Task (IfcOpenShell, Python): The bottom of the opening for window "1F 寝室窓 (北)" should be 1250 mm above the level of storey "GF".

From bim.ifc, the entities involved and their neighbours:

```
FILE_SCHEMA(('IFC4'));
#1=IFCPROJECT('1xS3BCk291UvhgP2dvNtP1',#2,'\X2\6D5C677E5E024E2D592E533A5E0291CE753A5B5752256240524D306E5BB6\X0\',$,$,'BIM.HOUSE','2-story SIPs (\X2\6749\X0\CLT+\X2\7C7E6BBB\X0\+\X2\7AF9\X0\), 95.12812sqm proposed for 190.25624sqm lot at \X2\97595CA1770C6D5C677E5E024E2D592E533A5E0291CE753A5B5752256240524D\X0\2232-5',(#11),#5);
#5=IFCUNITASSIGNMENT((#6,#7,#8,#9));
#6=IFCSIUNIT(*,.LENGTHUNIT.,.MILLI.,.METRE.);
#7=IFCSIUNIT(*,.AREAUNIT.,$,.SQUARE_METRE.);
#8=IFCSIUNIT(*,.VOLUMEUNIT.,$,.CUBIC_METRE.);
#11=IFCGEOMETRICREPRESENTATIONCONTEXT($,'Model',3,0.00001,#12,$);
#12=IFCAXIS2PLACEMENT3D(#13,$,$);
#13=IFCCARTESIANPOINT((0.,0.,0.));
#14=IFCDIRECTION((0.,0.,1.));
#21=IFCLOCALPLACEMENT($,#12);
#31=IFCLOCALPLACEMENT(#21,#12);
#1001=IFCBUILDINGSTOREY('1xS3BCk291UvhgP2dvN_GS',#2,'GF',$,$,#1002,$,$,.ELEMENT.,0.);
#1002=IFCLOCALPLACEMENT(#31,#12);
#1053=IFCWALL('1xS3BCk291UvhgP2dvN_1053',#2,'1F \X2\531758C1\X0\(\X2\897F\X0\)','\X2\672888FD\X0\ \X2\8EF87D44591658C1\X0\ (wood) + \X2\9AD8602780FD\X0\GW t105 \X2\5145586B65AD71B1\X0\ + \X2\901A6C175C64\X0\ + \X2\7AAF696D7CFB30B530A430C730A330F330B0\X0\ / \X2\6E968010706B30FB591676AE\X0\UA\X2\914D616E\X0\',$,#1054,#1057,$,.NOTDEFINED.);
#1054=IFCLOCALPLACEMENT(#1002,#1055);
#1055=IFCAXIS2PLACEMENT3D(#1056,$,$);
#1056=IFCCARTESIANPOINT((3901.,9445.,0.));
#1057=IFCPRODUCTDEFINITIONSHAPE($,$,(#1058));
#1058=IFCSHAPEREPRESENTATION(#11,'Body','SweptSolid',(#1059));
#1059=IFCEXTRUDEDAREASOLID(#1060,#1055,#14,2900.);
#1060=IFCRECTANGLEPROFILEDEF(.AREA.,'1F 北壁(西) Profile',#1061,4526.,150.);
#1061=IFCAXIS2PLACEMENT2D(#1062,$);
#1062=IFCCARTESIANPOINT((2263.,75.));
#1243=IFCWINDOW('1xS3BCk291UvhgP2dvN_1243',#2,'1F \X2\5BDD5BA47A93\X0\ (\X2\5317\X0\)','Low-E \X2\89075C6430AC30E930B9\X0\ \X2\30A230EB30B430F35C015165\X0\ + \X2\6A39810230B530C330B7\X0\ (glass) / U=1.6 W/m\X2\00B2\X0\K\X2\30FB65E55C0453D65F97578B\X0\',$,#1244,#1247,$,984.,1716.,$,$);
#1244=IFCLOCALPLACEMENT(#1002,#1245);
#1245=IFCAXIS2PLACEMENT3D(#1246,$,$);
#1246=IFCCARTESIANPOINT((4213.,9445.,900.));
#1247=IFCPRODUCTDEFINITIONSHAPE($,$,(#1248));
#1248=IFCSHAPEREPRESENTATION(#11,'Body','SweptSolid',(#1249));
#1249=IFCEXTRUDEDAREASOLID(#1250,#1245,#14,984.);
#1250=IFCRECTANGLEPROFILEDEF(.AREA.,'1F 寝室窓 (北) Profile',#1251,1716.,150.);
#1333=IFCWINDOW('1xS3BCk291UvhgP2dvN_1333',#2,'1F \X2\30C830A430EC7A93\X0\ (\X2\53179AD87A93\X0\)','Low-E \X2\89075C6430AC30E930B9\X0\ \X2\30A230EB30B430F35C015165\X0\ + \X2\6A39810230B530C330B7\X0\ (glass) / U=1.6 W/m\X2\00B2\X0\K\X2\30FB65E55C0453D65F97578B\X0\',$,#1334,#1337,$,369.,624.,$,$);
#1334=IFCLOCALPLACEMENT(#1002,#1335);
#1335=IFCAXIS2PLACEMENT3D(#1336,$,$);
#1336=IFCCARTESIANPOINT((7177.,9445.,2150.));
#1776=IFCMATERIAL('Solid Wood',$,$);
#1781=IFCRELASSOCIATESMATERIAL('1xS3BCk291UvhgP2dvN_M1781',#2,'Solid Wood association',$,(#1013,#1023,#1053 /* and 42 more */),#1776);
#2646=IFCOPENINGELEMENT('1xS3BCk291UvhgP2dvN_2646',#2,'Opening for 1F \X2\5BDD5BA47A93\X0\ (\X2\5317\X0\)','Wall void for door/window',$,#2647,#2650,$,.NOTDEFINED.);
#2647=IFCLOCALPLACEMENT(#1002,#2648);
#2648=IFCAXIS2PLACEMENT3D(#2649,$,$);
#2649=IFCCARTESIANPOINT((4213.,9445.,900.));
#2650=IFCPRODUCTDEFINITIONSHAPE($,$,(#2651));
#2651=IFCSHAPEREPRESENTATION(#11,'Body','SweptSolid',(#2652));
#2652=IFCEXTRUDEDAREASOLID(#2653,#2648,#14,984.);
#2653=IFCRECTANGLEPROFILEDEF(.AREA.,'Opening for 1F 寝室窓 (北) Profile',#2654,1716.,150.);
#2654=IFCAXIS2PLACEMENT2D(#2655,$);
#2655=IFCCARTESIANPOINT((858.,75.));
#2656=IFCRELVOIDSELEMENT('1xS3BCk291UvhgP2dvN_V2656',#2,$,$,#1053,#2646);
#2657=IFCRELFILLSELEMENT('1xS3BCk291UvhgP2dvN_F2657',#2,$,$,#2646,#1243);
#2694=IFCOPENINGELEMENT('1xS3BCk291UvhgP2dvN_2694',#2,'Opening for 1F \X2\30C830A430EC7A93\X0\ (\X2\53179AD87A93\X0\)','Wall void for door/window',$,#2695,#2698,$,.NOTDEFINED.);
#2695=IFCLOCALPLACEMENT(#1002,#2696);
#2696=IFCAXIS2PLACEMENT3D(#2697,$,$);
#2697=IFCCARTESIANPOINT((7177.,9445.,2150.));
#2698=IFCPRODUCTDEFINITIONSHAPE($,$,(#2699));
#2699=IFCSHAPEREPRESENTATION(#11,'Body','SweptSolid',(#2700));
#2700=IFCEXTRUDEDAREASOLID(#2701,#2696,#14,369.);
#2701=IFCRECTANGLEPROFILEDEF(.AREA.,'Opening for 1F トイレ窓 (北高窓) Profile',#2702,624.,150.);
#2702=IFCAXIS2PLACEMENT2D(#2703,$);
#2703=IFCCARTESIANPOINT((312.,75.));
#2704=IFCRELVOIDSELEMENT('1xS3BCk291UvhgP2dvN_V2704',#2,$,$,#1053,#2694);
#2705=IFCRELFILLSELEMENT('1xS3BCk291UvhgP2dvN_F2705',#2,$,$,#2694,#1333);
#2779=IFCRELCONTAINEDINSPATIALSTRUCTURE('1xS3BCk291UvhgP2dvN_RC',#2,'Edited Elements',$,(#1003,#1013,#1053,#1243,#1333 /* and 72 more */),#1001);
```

```python
import numpy as np
import ifcopenshell
import ifcopenshell.api.geometry
import ifcopenshell.geom
import ifcopenshell.util.element
import ifcopenshell.util.placement
import ifcopenshell.util.shape
import ifcopenshell.util.unit

model = ifcopenshell.open("bim.ifc")
unit_scale = ifcopenshell.util.unit.calculate_unit_scale(model)

window = model.by_guid("1xS3BCk291UvhgP2dvN_1243")
opening = window.FillsVoids[0].RelatingOpeningElement
storey = ifcopenshell.util.element.get_container(window, ifc_class="IfcBuildingStorey")
level = ifcopenshell.util.placement.get_local_placement(storey.ObjectPlacement)[2, 3]

# The opening's origin need not be at the sill, so measure its lowest point.
shape = ifcopenshell.geom.create_shape(ifcopenshell.geom.settings(), opening)
bottom = ifcopenshell.util.shape.get_shape_bottom_elevation(shape, shape.geometry) / unit_scale
dz = level + 1.25 / unit_scale - bottom

shift = np.array([0.0, 0.0, dz])
# The window is not placed relative to its opening, so move both.
for product in (opening, window):
    matrix = ifcopenshell.util.placement.get_local_placement(product.ObjectPlacement)
    matrix[:3, 3] += shift
    ifcopenshell.api.geometry.edit_object_placement(model, product=product, matrix=matrix, is_si=False)

print(f"moved by {dz * unit_scale:+.3f} m")

model.write("bim_v2.ifc")
```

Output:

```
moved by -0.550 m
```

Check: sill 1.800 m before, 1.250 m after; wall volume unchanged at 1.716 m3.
